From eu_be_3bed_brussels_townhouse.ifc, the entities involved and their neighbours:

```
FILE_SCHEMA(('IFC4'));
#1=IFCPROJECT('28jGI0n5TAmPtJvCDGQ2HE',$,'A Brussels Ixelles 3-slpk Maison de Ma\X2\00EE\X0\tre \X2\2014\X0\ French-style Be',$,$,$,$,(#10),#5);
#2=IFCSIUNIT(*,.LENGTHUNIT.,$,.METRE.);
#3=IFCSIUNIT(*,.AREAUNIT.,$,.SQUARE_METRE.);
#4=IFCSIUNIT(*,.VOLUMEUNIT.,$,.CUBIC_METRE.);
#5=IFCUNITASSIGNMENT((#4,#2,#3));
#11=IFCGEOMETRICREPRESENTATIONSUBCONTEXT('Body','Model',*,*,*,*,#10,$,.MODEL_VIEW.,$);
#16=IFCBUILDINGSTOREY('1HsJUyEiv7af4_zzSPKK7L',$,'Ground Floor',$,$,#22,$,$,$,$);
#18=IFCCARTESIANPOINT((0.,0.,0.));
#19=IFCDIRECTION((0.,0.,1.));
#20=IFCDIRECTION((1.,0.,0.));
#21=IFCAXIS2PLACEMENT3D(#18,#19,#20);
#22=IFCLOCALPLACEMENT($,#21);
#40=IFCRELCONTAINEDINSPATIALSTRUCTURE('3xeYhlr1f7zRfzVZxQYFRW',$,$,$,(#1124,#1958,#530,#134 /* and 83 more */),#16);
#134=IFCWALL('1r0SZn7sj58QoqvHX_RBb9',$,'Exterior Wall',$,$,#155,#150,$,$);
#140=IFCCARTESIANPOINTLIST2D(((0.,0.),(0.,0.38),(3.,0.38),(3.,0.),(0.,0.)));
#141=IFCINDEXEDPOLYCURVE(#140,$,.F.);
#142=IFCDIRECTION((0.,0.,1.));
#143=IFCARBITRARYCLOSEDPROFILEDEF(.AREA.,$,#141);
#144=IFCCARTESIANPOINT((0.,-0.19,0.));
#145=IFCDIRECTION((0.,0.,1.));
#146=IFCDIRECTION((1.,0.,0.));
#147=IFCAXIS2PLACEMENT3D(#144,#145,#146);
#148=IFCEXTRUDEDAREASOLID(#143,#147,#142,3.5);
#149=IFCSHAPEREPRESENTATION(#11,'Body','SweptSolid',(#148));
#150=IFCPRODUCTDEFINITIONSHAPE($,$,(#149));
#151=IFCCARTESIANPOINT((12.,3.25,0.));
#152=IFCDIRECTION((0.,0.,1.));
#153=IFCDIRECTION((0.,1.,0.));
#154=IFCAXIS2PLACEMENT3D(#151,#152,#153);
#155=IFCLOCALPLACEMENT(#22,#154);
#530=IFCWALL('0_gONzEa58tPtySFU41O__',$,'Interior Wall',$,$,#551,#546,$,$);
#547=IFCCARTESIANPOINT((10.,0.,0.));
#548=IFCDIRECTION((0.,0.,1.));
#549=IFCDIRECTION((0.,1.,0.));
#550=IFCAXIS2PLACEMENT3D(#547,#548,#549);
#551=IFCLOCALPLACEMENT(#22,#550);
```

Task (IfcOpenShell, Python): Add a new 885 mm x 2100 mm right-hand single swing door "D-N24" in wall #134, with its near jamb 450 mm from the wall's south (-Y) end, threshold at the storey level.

```python
import numpy as np
import ifcopenshell
import ifcopenshell.api.feature
import ifcopenshell.api.geometry
import ifcopenshell.api.root
import ifcopenshell.api.spatial
import ifcopenshell.geom
import ifcopenshell.util.element
import ifcopenshell.util.placement
import ifcopenshell.util.representation
import ifcopenshell.util.shape
import ifcopenshell.util.unit

model = ifcopenshell.open("eu_be_3bed_brussels_townhouse.ifc")
unit_scale = ifcopenshell.util.unit.calculate_unit_scale(model)
settings = ifcopenshell.geom.settings()


def volume(element):
    """Net volume in cubic metres, openings subtracted."""
    shape = ifcopenshell.geom.create_shape(settings, element)
    return ifcopenshell.util.shape.get_volume(shape.geometry)


wall = model.by_guid("1r0SZn7sj58QoqvHX_RBb9")
storey = ifcopenshell.util.element.get_container(wall, ifc_class="IfcBuildingStorey")
context = ifcopenshell.util.representation.get_context(model, "Model", "Body", "MODEL_VIEW")
before = volume(wall)

width, height, from_end, sill = 0.885, 2.1, 0.45, 0.0  # metres

# The wall runs along its own X axis, and the end named is its -X end.
wall_shape = ifcopenshell.geom.create_shape(settings, wall)
x, y, z = ifcopenshell.util.shape.get_vertices(wall_shape.geometry).T
start = x.min() + from_end
face, thickness = float(y.min()), float(y.max() - y.min())
wall_matrix = ifcopenshell.util.placement.get_local_placement(wall.ObjectPlacement)
level = ifcopenshell.util.placement.get_local_placement(storey.ObjectPlacement)[2, 3]


def in_wall(x, y):
    """Placement at x, y metres in the wall's axes, at sill height."""
    matrix = wall_matrix.copy()
    matrix[:, 3] = wall_matrix @ np.array([x / unit_scale, y / unit_scale, 0.0, 1.0])
    matrix[2, 3] = level + sill / unit_scale
    return matrix


# Opening: a box that overshoots both wall faces by 50 mm.
opening = ifcopenshell.api.root.create_entity(model, ifc_class="IfcOpeningElement", predefined_type="OPENING")
box = ifcopenshell.api.geometry.add_wall_representation(
    model, context=context, length=width, height=height, thickness=thickness + 0.1
)
ifcopenshell.api.geometry.assign_representation(model, product=opening, representation=box)
ifcopenshell.api.geometry.edit_object_placement(model, product=opening, matrix=in_wall(start, face - 0.05), is_si=False)
ifcopenshell.api.feature.add_feature(model, feature=opening, element=wall)

door = ifcopenshell.api.root.create_entity(model, ifc_class="IfcDoor", name="D-N24", predefined_type="DOOR")
door.OverallWidth, door.OverallHeight = width / unit_scale, height / unit_scale
door.OperationType = "SINGLE_SWING_RIGHT"
body = ifcopenshell.api.geometry.add_door_representation(
    model,
    context=context,
    overall_width=door.OverallWidth,
    overall_height=door.OverallHeight,
    operation_type="SINGLE_SWING_RIGHT",
    lining_properties={"LiningDepth": thickness / unit_scale, "ThresholdDepth": thickness / unit_scale},
)
ifcopenshell.api.geometry.assign_representation(model, product=door, representation=body)
ifcopenshell.api.spatial.assign_container(model, products=[door], relating_structure=storey)
ifcopenshell.api.feature.add_filling(model, opening=opening, element=door)

# The lining spans the wall, so the door starts at the wall face.
ifcopenshell.api.geometry.edit_object_placement(model, product=door, matrix=in_wall(start, face), is_si=False)

after = volume(wall)

print(f"wall volume {before:.3f} -> {after:.3f} m3")

model.write("eu_be_3bed_brussels_townhouse_edited.ifc")
```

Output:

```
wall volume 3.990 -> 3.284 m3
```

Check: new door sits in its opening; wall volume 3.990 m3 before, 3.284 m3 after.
